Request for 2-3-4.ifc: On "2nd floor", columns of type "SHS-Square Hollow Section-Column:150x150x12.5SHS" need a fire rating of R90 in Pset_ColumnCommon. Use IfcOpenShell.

First a look at what the model holds.

```python
import ifcopenshell
import ifcopenshell.util.element

model = ifcopenshell.open("2-3-4.ifc")
print(model.schema)
storey = next(s for s in model.by_type("IfcBuildingStorey") if s.Name == "2nd floor")
columns = [e for e in ifcopenshell.util.element.get_decomposition(storey) if e.is_a("IfcColumn")]
seen = {}
for e in columns:
    element_type = ifcopenshell.util.element.get_type(e)
    key = (element_type.Name if element_type != e and element_type else None, ifcopenshell.util.element.get_pset(e, "Pset_ColumnCommon", "FireRating"))
    seen[key] = seen.get(key, 0) + 1
for (name, value), count in sorted(seen.items(), key=str):
    print(count, "x", name, "|", value)
```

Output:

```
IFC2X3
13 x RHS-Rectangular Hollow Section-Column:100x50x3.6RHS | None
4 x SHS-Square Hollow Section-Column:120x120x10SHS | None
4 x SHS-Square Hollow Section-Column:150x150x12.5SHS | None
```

```python
import ifcopenshell
import ifcopenshell.api.pset
import ifcopenshell.util.element

model = ifcopenshell.open("2-3-4.ifc")

storey = next(s for s in model.by_type("IfcBuildingStorey") if s.Name == "2nd floor")
columns = [e for e in ifcopenshell.util.element.get_decomposition(storey) if e.is_a("IfcColumn")]

count = 0
for e in columns:
    element_type = ifcopenshell.util.element.get_type(e)
    if element_type in (None, e) or element_type.Name != "SHS-Square Hollow Section-Column:150x150x12.5SHS":
        continue
    # add_pset returns the element's existing set when there is one.
    pset = ifcopenshell.api.pset.add_pset(model, product=e, name="Pset_ColumnCommon")
    ifcopenshell.api.pset.edit_pset(model, pset=pset, properties={"FireRating": "R90"})
    count += 1

print(count, "columns updated")

model.write("2-3-4_v2.ifc")
```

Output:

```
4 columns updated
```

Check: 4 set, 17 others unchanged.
